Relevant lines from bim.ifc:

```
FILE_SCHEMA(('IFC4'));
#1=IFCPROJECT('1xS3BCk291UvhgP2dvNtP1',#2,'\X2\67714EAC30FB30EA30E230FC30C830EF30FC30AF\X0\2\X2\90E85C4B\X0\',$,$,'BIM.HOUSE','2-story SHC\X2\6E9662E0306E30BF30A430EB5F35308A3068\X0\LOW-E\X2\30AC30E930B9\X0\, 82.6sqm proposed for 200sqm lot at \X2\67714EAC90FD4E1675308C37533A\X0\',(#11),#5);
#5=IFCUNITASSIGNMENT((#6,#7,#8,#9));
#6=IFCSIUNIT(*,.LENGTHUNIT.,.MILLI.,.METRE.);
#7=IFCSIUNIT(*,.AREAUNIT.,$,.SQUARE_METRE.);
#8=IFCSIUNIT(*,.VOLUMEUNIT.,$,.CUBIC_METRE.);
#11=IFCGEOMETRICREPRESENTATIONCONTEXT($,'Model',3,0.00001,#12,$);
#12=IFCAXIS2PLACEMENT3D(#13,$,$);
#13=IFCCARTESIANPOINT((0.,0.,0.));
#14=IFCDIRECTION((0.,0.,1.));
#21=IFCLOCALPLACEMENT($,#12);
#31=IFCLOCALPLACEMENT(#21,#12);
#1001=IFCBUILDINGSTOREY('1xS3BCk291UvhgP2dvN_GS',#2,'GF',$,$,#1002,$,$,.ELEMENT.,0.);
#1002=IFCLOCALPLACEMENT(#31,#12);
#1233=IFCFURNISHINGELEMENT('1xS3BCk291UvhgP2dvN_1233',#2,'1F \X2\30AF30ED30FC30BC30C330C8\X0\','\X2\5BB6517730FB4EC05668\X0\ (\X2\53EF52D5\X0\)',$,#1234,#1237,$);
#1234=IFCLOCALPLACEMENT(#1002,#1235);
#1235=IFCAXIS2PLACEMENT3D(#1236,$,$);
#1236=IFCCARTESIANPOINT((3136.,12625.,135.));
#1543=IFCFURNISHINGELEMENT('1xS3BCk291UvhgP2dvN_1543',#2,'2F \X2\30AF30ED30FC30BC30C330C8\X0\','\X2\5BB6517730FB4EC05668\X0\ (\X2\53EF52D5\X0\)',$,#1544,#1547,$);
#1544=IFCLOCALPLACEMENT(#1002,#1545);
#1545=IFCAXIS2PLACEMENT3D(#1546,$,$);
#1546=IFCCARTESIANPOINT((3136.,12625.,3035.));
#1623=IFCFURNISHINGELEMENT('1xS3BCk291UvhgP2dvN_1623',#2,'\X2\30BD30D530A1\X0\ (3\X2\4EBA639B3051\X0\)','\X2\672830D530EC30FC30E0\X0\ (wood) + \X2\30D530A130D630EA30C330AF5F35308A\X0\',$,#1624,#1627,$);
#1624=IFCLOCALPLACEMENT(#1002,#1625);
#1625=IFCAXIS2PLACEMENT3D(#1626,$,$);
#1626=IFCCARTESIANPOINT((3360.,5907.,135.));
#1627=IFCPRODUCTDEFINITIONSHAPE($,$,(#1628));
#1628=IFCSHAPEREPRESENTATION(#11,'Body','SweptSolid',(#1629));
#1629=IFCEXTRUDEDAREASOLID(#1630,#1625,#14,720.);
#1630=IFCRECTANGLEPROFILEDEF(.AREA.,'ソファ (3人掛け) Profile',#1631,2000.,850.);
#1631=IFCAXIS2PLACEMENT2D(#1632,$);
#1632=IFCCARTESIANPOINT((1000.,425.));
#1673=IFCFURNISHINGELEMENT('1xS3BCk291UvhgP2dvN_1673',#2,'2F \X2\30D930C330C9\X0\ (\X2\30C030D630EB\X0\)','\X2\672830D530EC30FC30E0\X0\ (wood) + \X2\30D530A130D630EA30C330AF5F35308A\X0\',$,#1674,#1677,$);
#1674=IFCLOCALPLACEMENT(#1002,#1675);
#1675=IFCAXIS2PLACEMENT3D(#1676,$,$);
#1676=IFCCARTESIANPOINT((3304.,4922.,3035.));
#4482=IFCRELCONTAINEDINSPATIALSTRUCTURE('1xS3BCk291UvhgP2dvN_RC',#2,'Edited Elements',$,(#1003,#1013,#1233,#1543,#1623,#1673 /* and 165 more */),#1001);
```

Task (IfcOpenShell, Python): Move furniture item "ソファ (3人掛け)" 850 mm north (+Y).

```python
import ifcopenshell
import ifcopenshell.api.geometry
import ifcopenshell.util.placement

model = ifcopenshell.open("bim.ifc")

item = model.by_guid("1xS3BCk291UvhgP2dvN_1623")
matrix = ifcopenshell.util.placement.get_local_placement(item.ObjectPlacement)
matrix[1, 3] += 850.0
ifcopenshell.api.geometry.edit_object_placement(model, product=item, matrix=matrix, is_si=False)

print(ifcopenshell.util.placement.get_local_placement(item.ObjectPlacement).round(3) + 0.0)

model.write("bim_v2.ifc")
```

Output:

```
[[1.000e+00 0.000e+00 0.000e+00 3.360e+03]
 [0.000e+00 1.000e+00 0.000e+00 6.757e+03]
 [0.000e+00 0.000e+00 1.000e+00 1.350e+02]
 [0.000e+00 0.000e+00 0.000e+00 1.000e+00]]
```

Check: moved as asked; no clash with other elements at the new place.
